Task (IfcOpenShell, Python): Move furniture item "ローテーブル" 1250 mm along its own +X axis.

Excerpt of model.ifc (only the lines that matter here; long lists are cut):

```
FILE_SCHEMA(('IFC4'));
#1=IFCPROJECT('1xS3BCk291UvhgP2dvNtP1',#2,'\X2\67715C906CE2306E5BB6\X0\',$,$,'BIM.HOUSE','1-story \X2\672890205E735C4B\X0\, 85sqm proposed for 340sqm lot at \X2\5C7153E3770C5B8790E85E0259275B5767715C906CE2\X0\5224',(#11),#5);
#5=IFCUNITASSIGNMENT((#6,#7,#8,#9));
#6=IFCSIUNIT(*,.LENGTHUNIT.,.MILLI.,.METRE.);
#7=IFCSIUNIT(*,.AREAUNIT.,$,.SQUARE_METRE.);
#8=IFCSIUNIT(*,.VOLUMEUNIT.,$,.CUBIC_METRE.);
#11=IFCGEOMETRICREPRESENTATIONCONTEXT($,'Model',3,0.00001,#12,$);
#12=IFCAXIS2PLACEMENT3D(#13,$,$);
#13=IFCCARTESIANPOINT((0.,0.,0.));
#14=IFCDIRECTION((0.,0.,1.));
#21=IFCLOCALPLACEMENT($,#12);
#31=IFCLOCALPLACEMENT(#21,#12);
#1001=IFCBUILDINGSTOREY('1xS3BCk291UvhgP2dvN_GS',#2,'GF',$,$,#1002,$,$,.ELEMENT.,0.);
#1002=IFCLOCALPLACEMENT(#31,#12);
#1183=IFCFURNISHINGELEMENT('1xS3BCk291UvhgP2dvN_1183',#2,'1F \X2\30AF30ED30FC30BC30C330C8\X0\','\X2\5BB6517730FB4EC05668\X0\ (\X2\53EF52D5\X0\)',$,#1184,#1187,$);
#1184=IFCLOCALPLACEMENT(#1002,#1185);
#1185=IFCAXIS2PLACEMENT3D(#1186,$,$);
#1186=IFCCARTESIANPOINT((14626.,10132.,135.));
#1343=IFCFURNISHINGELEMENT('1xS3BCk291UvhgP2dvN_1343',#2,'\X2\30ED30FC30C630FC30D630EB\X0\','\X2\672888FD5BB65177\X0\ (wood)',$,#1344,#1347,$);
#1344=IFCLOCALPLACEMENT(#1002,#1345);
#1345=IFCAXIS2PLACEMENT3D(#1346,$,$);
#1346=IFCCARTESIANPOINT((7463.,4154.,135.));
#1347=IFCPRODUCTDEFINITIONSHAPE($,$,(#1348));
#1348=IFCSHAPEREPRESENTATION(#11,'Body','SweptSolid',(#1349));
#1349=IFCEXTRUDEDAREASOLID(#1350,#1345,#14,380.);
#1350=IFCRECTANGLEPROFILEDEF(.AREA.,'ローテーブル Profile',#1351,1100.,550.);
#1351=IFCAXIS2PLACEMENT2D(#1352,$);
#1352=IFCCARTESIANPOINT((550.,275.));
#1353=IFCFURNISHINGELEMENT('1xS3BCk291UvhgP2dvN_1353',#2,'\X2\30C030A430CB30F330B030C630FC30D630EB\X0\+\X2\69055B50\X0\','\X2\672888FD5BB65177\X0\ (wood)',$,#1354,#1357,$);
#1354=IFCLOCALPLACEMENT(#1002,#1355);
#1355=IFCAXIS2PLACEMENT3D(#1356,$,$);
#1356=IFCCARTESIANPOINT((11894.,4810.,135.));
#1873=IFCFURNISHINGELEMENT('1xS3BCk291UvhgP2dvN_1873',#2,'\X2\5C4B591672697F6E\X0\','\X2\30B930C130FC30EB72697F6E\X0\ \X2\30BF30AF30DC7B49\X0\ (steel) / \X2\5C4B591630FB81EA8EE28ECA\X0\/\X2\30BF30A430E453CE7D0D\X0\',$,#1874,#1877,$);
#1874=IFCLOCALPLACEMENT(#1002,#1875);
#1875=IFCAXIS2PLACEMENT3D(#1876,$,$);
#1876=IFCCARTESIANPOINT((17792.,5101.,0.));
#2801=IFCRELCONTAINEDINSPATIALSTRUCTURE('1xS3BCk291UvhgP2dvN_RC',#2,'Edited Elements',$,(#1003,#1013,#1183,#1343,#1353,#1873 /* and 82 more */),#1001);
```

```python
import ifcopenshell
import ifcopenshell.api.geometry
import ifcopenshell.util.placement

model = ifcopenshell.open("model.ifc")

item = model.by_guid("1xS3BCk291UvhgP2dvN_1343")
matrix = ifcopenshell.util.placement.get_local_placement(item.ObjectPlacement)
matrix[:3, 3] += matrix[:3, 0] * 1250.0
ifcopenshell.api.geometry.edit_object_placement(model, product=item, matrix=matrix, is_si=False)

print(ifcopenshell.util.placement.get_local_placement(item.ObjectPlacement).round(3) + 0.0)

model.write("model_v2.ifc")
```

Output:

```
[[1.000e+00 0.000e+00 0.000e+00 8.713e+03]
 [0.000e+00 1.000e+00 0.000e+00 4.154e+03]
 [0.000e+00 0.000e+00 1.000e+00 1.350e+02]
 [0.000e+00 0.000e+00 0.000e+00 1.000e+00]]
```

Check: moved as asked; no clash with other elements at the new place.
